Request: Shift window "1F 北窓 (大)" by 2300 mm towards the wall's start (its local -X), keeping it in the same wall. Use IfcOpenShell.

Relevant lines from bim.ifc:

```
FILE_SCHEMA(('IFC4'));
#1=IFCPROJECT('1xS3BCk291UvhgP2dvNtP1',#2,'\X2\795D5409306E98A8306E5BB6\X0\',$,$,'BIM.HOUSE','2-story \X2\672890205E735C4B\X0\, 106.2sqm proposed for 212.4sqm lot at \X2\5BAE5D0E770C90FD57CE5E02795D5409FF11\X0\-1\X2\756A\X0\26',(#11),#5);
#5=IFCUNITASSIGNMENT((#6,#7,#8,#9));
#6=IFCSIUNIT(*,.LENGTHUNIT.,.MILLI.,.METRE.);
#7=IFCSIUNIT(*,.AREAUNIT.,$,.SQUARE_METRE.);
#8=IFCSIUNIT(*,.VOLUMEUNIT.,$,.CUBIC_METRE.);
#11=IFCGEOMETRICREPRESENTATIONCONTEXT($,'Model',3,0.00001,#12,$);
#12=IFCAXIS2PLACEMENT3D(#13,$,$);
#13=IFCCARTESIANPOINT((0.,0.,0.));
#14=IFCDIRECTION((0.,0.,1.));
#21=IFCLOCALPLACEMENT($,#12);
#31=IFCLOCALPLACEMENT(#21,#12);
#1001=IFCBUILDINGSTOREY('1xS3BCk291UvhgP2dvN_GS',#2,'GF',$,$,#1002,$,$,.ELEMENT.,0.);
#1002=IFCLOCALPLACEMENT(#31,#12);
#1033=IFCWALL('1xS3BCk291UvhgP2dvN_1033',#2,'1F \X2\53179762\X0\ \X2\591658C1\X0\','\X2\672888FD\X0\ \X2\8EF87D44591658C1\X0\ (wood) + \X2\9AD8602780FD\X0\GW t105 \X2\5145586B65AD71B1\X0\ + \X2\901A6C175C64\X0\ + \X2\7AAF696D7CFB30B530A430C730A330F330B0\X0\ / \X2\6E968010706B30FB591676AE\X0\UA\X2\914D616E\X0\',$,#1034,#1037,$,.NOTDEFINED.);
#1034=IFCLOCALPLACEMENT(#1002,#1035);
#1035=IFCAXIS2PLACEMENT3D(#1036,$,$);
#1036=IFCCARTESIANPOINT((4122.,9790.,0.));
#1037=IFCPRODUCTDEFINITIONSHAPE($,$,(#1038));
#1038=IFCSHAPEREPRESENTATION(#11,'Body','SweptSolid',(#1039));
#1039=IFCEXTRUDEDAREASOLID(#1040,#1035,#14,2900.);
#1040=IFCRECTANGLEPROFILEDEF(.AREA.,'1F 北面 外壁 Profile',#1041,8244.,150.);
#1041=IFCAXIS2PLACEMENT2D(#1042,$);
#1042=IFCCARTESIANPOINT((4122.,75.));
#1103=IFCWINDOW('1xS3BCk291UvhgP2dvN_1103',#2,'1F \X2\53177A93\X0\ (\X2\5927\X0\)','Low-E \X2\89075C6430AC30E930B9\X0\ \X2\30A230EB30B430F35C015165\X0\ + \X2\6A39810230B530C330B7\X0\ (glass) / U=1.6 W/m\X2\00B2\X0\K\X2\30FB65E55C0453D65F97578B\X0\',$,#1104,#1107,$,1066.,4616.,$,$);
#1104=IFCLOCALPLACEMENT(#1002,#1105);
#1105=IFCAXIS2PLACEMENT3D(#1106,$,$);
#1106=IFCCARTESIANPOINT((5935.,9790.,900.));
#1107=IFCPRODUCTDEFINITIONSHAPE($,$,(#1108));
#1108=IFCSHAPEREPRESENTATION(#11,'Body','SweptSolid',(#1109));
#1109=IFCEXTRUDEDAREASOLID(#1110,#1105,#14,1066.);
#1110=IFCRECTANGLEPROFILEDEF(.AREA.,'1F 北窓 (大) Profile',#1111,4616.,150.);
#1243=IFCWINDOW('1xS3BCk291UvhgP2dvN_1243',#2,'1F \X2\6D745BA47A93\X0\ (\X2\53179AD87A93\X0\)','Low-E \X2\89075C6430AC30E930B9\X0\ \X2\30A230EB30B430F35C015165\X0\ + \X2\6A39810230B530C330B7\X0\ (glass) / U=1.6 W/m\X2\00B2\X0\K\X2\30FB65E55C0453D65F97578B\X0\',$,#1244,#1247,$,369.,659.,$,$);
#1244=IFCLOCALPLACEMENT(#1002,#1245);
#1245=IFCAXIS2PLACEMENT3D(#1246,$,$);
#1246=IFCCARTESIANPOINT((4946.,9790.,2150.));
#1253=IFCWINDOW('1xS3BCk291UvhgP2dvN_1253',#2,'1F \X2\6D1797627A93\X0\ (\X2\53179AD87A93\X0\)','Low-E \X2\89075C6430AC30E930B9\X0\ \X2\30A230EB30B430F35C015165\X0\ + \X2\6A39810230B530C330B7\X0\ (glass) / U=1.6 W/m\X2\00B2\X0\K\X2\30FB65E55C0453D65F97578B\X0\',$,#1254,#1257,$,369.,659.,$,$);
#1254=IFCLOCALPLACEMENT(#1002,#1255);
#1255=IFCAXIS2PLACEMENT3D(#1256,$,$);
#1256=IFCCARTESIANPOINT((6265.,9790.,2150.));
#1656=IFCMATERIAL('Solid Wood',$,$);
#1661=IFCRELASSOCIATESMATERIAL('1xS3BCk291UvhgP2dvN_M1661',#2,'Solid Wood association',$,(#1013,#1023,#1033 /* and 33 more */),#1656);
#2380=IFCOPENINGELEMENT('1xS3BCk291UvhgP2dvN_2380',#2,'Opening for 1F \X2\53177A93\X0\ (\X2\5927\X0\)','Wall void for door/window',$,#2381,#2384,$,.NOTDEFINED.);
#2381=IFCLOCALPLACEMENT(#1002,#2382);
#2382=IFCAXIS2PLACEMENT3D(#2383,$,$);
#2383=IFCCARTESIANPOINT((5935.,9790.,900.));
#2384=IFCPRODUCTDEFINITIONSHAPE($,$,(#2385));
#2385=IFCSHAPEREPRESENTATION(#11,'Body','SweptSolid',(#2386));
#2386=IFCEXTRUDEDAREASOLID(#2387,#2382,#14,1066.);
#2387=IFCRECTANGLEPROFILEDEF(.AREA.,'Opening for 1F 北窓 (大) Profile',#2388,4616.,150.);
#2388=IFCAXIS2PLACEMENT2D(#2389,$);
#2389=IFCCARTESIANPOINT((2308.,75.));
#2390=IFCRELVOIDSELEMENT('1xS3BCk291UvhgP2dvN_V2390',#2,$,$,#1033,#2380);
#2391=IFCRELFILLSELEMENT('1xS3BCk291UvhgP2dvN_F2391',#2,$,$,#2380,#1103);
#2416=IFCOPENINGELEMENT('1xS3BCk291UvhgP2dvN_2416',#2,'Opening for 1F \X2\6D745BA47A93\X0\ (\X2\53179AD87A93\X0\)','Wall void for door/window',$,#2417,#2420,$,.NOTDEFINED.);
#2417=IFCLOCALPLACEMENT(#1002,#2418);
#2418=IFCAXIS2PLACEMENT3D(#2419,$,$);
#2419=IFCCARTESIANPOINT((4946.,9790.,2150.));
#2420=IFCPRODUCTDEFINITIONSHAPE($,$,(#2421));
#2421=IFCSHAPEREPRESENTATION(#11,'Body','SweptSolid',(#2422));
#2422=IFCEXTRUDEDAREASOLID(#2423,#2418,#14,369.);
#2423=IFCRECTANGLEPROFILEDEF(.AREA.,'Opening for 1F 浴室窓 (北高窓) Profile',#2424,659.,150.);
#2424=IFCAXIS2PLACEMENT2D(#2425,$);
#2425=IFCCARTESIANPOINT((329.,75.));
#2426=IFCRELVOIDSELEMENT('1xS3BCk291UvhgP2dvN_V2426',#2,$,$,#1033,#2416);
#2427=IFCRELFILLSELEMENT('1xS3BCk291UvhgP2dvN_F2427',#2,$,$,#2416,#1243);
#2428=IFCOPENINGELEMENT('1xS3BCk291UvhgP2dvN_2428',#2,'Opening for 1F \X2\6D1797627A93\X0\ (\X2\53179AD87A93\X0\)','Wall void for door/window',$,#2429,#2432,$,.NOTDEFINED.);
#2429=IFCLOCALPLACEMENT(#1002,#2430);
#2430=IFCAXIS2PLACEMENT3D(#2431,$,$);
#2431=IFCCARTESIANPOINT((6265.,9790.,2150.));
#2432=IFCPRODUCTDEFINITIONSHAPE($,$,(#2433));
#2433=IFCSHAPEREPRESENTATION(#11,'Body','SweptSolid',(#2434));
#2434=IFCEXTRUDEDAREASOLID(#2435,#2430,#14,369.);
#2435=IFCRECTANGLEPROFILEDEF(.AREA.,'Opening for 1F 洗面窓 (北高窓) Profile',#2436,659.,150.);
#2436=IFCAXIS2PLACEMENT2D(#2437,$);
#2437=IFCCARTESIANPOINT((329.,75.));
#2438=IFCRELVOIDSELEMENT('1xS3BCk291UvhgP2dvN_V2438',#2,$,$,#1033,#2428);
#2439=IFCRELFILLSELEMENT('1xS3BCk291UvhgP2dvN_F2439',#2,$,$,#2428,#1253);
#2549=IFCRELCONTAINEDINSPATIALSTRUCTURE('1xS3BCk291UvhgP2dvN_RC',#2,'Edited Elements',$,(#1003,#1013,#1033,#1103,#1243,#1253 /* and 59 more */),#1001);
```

```python
import ifcopenshell
import ifcopenshell.api.geometry
import ifcopenshell.util.placement
import ifcopenshell.util.unit

model = ifcopenshell.open("bim.ifc")
unit_scale = ifcopenshell.util.unit.calculate_unit_scale(model)

window = model.by_guid("1xS3BCk291UvhgP2dvN_1103")
opening = window.FillsVoids[0].RelatingOpeningElement
wall = opening.VoidsElements[0].RelatingBuildingElement

wall_matrix = ifcopenshell.util.placement.get_local_placement(wall.ObjectPlacement)
shift = wall_matrix[:3, 0] * -2.3 / unit_scale
before = ifcopenshell.util.placement.get_local_placement(window.ObjectPlacement)[:3, 3].copy()

# The window is not placed relative to its opening, so move both.
for product in (opening, window):
    matrix = ifcopenshell.util.placement.get_local_placement(product.ObjectPlacement)
    matrix[:3, 3] += shift
    ifcopenshell.api.geometry.edit_object_placement(model, product=product, matrix=matrix, is_si=False)

after = ifcopenshell.util.placement.get_local_placement(window.ObjectPlacement)[:3, 3]
print("window moved by", (after - before).round(3) + 0.0)

model.write("bim_v2.ifc")
```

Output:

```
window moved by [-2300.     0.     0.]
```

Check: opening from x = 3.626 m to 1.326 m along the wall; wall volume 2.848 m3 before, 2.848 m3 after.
